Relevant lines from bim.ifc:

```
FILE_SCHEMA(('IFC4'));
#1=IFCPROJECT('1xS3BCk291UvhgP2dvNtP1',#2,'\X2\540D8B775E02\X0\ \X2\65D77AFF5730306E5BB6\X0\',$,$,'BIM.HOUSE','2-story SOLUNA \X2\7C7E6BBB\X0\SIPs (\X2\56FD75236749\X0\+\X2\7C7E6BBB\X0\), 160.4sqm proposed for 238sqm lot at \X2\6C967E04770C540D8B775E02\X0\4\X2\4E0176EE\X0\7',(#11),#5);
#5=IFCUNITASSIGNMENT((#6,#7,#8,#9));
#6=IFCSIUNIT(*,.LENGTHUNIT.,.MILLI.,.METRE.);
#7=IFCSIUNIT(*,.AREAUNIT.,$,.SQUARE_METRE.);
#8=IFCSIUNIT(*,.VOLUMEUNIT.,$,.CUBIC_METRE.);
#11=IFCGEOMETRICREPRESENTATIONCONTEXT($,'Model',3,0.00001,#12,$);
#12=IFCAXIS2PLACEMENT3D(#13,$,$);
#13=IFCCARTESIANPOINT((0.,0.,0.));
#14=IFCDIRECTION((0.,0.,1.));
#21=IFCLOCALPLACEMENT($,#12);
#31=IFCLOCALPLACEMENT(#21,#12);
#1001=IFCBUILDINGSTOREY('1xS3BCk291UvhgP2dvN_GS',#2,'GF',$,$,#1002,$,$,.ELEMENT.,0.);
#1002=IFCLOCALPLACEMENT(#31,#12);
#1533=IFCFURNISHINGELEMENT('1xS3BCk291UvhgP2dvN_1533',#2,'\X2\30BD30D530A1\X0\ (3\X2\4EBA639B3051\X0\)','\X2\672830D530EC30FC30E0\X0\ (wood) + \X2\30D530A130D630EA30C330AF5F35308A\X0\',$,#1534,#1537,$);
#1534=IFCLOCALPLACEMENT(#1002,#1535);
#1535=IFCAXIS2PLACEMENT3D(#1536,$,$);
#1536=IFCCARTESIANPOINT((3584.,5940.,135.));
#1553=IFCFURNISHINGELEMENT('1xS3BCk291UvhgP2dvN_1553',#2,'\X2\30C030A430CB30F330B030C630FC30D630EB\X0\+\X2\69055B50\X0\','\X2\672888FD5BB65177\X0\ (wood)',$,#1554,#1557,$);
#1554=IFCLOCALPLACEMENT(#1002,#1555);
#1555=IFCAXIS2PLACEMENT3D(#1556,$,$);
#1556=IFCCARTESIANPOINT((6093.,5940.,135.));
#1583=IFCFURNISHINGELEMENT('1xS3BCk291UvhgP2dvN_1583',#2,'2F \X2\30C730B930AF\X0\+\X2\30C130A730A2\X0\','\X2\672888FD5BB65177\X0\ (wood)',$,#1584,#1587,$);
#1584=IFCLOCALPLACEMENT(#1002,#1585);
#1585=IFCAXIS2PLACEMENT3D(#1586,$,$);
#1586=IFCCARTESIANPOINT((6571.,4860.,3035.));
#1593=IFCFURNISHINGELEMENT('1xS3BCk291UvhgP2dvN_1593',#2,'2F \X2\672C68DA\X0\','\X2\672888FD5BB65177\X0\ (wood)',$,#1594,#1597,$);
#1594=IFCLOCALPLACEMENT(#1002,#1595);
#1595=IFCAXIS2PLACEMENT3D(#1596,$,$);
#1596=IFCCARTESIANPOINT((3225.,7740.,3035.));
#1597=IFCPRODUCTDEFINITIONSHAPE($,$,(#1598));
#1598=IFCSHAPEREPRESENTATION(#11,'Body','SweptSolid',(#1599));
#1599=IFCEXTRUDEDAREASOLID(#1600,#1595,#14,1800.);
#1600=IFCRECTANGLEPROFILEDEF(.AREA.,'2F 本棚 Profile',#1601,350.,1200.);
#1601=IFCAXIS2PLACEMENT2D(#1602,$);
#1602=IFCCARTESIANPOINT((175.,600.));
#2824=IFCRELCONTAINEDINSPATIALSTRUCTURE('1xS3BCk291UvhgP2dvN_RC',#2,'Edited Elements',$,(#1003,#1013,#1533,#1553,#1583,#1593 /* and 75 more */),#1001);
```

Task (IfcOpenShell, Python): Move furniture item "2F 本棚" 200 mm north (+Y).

```python
import ifcopenshell
import ifcopenshell.api.geometry
import ifcopenshell.util.placement
import ifcopenshell.util.unit

model = ifcopenshell.open("bim.ifc")
unit_scale = ifcopenshell.util.unit.calculate_unit_scale(model)

item = model.by_guid("1xS3BCk291UvhgP2dvN_1593")
matrix = ifcopenshell.util.placement.get_local_placement(item.ObjectPlacement)
matrix[1, 3] += 0.2 / unit_scale
ifcopenshell.api.geometry.edit_object_placement(model, product=item, matrix=matrix, is_si=False)

print(ifcopenshell.util.placement.get_local_placement(item.ObjectPlacement).round(3) + 0.0)

model.write("bim_edited.ifc")
```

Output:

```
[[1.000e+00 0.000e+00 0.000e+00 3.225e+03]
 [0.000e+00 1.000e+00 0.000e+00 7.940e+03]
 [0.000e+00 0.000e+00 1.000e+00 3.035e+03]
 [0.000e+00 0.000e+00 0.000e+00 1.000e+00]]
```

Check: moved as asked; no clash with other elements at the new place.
